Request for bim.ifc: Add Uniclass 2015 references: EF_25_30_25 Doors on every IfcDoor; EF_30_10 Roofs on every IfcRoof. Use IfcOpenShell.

First a look at what the model holds.

```python
import ifcopenshell

model = ifcopenshell.open("bim.ifc")
print(model.schema)
print("classifications:", [c.Name for c in model.by_type("IfcClassification")])
for ifc_class in ("IfcDoor", "IfcRoof", "IfcStair", "IfcWall", "IfcWindow"):
    print(ifc_class, len(model.by_type(ifc_class)))
```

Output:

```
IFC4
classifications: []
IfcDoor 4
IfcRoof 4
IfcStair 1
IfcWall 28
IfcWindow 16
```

```python
import ifcopenshell
import ifcopenshell.api.classification

model = ifcopenshell.open("bim.ifc")

system = ifcopenshell.api.classification.add_classification(model, classification="Uniclass 2015")

codes = {
    "IfcDoor": ("EF_25_30_25", "Doors"),
    "IfcRoof": ("EF_30_10", "Roofs"),
}
for ifc_class, (code, name) in codes.items():
    products = model.by_type(ifc_class)
    ifcopenshell.api.classification.add_reference(
        model, products=products, classification=system, identification=code, name=name
    )
    print(code, len(products))

model.write("bim_updated.ifc")
```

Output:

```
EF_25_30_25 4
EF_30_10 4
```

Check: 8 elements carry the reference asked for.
